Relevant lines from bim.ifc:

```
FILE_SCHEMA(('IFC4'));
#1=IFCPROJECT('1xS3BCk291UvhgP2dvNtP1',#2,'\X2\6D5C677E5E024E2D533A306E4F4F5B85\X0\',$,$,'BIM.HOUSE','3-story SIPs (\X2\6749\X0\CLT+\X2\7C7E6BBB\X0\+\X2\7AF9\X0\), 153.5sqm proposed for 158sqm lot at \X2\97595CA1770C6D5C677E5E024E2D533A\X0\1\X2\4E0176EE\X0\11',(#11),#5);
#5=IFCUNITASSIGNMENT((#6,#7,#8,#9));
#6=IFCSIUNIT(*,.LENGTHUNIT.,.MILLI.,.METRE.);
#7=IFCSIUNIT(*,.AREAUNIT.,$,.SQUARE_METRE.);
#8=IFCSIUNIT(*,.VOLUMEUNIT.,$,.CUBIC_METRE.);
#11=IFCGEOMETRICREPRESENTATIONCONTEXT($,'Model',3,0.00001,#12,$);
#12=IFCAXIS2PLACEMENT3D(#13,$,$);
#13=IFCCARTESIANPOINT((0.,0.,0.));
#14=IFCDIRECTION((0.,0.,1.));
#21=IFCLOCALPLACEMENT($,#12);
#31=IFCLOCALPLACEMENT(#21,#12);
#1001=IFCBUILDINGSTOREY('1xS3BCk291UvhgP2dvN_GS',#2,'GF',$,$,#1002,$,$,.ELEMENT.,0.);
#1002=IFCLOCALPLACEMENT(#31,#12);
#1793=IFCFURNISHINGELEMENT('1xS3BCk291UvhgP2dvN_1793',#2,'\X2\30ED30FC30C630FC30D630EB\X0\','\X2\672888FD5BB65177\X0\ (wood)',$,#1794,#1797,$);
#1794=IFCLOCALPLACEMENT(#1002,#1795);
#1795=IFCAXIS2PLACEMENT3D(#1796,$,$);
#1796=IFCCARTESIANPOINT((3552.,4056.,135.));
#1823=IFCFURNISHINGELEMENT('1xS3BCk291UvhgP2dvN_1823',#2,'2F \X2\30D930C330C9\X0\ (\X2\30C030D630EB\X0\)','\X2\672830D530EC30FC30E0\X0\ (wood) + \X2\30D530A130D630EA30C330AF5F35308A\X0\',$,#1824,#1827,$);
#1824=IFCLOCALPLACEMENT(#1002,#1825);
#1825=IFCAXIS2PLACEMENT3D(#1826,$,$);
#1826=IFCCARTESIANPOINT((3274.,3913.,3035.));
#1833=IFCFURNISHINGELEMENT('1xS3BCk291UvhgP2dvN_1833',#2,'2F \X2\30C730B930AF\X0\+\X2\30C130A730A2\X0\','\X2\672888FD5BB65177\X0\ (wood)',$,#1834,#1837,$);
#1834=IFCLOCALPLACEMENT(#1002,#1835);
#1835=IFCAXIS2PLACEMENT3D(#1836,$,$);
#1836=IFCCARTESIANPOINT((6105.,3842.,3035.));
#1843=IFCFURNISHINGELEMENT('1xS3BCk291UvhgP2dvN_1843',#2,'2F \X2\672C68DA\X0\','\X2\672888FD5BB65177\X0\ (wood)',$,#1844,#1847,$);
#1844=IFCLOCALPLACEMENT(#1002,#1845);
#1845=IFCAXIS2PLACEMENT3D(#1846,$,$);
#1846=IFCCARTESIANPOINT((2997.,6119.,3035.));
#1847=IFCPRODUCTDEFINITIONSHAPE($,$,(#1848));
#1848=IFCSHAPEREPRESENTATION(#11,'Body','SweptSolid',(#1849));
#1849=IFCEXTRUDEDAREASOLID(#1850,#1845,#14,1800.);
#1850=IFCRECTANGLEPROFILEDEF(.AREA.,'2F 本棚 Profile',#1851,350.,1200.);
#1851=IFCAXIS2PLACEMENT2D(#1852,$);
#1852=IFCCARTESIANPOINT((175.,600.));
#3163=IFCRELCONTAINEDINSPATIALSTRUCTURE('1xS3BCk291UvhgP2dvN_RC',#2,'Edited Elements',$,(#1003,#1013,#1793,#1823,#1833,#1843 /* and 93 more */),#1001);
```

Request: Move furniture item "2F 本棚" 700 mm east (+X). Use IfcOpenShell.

```python
import ifcopenshell
import ifcopenshell.api.geometry
import ifcopenshell.util.placement

model = ifcopenshell.open("bim.ifc")

item = model.by_guid("1xS3BCk291UvhgP2dvN_1843")
matrix = ifcopenshell.util.placement.get_local_placement(item.ObjectPlacement)
matrix[0, 3] += 700.0
ifcopenshell.api.geometry.edit_object_placement(model, product=item, matrix=matrix, is_si=False)

print(ifcopenshell.util.placement.get_local_placement(item.ObjectPlacement).round(3) + 0.0)

model.write("bim-out.ifc")
```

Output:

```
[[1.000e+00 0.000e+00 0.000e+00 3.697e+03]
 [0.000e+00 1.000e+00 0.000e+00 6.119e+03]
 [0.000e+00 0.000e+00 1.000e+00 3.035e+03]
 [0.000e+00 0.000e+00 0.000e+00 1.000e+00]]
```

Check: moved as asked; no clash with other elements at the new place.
